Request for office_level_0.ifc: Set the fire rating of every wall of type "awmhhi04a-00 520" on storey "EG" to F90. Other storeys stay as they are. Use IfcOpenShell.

First a look at what the model holds.

```python
import ifcopenshell
import ifcopenshell.util.element

model = ifcopenshell.open("office_level_0.ifc")
print(model.schema)
storey = next(s for s in model.by_type("IfcBuildingStorey") if s.Name == "EG")
walls = [e for e in ifcopenshell.util.element.get_decomposition(storey) if e.is_a("IfcWall")]
seen = {}
for e in walls:
    element_type = ifcopenshell.util.element.get_type(e)
    key = (element_type.Name if element_type != e and element_type else None, ifcopenshell.util.element.get_pset(e, "Pset_WallCommon", "FireRating"))
    seen[key] = seen.get(key, 0) + 1
for (name, value), count in sorted(seen.items(), key=str):
    print(count, "x", name, "|", value)
```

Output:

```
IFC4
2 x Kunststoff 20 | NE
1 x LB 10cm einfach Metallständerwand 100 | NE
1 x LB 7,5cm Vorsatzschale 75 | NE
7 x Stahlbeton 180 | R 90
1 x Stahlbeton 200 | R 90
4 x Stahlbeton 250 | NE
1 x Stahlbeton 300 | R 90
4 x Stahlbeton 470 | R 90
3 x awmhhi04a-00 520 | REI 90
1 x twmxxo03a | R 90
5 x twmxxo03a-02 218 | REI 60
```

```python
import ifcopenshell
import ifcopenshell.api.pset
import ifcopenshell.util.element

model = ifcopenshell.open("office_level_0.ifc")

storey = next(s for s in model.by_type("IfcBuildingStorey") if s.Name == "EG")
walls = [e for e in ifcopenshell.util.element.get_decomposition(storey) if e.is_a("IfcWall")]

count = 0
for e in walls:
    element_type = ifcopenshell.util.element.get_type(e)
    if element_type in (None, e) or element_type.Name != "awmhhi04a-00 520":
        continue
    # add_pset returns the element's existing set when there is one.
    pset = ifcopenshell.api.pset.add_pset(model, product=e, name="Pset_WallCommon")
    ifcopenshell.api.pset.edit_pset(model, pset=pset, properties={"FireRating": "F90"})
    count += 1

print(count, "walls updated")

model.write("office_level_0_updated.ifc")
```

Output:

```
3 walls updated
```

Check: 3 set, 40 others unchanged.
